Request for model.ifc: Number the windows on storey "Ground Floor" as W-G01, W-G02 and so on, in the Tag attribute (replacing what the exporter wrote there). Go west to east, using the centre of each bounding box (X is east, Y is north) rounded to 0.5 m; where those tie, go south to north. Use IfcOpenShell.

First a look at what the model holds.

```python
import ifcopenshell
import ifcopenshell.util.element
import ifcopenshell.util.placement

model = ifcopenshell.open("model.ifc")
print(model.schema)
storey = next(s for s in model.by_type("IfcBuildingStorey") if s.Name == "Ground Floor")
windows = [e for e in ifcopenshell.util.element.get_decomposition(storey) if e.is_a("IfcWindow")]
for e in sorted(windows, key=lambda e: e.id()):
    origin = ifcopenshell.util.placement.get_local_placement(e.ObjectPlacement)[:3, 3]
    print(e.id(), e.Tag, e.Name, origin.round(2) + 0.0, sep=" | ")
```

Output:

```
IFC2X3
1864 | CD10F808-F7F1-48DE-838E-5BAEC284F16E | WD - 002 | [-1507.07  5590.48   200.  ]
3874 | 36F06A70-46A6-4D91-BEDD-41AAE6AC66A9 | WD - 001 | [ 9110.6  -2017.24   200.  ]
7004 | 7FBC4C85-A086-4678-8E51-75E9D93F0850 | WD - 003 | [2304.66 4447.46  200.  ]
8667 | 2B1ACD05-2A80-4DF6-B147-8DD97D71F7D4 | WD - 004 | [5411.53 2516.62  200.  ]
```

```python
import ifcopenshell
import ifcopenshell.geom
import ifcopenshell.util.element
import ifcopenshell.util.shape

model = ifcopenshell.open("model.ifc")
settings = ifcopenshell.geom.settings()
settings.set("use-world-coords", True)


def centre(element):
    shape = ifcopenshell.geom.create_shape(settings, element)
    return ifcopenshell.util.shape.get_bbox_centroid(shape.geometry)


storey = next(s for s in model.by_type("IfcBuildingStorey") if s.Name == "Ground Floor")
windows = [e for e in ifcopenshell.util.element.get_decomposition(storey) if e.is_a("IfcWindow")]

# Insertion points can sit at a corner or the storey origin, so sort by the geometry (in metres).
centres = {e: centre(e) for e in windows}
windows.sort(key=lambda e: (round(centres[e][0] / 0.5), centres[e][1]))

for i, e in enumerate(windows, start=1):
    number = f"W-G{i:02d}"
    e.Tag = number
    print(e.id(), number)

model.write("model_updated.ifc")
```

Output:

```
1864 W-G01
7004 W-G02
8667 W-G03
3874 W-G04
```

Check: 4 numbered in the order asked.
